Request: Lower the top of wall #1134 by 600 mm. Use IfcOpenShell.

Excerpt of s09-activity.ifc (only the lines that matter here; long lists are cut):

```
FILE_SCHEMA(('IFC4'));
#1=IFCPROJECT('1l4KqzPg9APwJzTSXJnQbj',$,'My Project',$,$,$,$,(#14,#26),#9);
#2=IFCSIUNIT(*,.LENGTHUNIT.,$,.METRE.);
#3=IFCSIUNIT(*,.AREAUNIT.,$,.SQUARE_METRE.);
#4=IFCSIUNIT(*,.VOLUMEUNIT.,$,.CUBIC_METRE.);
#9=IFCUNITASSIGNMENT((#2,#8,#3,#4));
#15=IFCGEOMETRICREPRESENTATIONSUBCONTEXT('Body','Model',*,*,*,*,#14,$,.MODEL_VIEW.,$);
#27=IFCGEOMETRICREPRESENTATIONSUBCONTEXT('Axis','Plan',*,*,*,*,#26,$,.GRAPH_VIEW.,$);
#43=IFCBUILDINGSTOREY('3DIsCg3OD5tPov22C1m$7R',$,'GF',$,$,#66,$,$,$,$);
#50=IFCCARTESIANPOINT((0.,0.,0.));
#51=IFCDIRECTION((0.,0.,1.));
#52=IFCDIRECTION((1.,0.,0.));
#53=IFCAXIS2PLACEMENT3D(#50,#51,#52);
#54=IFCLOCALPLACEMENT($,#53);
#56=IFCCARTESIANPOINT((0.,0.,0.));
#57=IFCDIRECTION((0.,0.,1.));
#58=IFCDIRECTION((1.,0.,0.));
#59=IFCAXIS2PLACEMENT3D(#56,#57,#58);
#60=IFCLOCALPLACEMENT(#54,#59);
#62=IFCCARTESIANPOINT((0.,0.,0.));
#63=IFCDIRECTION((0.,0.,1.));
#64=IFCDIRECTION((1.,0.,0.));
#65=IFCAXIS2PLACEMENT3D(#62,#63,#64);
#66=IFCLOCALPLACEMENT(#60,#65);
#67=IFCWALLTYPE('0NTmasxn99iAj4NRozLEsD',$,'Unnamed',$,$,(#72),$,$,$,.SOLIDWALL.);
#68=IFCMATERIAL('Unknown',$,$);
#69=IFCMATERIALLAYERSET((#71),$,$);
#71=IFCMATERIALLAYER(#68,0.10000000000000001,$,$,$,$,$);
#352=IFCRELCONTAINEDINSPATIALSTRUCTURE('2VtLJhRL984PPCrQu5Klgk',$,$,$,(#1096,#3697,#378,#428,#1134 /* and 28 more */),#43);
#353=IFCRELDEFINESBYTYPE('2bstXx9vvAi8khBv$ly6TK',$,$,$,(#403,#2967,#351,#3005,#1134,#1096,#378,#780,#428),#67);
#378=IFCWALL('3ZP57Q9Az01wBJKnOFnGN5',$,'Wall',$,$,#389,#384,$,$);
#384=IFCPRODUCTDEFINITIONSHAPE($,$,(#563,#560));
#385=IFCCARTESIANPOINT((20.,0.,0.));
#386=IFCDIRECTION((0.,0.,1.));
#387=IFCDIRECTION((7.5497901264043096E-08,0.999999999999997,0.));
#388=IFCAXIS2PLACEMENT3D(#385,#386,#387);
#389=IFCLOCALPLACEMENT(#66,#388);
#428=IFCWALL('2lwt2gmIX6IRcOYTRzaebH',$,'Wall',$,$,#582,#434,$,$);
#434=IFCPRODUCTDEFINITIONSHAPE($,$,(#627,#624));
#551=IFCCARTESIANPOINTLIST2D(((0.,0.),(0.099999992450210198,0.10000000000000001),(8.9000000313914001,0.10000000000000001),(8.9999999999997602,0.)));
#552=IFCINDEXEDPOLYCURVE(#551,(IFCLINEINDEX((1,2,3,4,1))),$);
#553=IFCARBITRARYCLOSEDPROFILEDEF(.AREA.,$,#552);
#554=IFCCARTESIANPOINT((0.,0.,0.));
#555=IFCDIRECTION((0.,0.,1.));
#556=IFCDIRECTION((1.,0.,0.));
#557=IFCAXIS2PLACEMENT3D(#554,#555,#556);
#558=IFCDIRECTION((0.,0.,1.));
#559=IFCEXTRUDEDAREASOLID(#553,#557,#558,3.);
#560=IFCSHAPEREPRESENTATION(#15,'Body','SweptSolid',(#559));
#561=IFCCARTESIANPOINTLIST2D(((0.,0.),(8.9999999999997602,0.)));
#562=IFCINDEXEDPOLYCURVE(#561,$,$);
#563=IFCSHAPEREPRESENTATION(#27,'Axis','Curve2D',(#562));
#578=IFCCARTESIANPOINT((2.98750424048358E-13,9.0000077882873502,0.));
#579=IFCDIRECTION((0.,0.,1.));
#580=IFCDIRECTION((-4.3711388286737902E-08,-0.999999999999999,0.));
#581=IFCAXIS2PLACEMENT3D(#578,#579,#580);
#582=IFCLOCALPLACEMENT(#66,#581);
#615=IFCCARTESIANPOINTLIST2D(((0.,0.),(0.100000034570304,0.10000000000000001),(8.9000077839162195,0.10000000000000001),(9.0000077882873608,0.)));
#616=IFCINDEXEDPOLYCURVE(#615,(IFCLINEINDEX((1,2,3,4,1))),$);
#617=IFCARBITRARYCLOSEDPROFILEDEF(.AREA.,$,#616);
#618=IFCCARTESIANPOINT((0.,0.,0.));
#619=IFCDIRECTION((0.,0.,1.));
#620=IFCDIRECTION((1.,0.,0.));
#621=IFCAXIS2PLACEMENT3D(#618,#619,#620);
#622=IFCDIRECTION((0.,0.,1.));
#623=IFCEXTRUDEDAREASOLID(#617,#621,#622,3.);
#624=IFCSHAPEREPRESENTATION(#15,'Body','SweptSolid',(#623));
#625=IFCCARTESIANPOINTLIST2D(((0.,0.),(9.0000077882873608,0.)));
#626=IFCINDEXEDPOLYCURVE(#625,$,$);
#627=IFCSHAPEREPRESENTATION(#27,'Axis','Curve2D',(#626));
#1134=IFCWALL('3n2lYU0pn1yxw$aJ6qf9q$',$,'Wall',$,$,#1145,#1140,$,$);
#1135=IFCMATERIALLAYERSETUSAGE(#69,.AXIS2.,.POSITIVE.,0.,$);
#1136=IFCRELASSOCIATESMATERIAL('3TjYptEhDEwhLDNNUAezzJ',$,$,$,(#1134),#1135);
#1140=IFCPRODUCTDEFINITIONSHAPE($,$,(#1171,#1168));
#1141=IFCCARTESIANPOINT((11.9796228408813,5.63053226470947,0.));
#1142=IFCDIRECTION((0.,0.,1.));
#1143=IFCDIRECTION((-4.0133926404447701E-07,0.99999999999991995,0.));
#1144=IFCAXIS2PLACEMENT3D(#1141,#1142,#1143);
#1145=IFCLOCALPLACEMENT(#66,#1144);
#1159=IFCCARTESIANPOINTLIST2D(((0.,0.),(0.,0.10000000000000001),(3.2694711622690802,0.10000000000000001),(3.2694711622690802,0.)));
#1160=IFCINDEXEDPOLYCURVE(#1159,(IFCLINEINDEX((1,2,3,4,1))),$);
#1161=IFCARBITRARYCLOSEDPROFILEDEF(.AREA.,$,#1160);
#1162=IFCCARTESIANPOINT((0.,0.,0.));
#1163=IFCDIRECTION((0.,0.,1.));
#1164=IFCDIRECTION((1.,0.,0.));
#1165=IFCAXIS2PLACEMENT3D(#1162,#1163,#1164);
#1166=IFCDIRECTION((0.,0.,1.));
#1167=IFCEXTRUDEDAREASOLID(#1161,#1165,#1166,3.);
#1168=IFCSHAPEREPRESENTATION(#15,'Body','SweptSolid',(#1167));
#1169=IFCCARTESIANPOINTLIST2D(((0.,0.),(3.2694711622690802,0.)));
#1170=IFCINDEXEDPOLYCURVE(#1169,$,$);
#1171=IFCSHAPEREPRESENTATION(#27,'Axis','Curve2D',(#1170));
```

```python
import ifcopenshell
import ifcopenshell.geom
import ifcopenshell.util.representation
import ifcopenshell.util.shape

model = ifcopenshell.open("s09-activity.ifc")
settings = ifcopenshell.geom.settings()


def volume(element):
    """Net volume in cubic metres, openings subtracted."""
    shape = ifcopenshell.geom.create_shape(settings, element)
    return ifcopenshell.util.shape.get_volume(shape.geometry)


wall = model.by_guid("3n2lYU0pn1yxw$aJ6qf9q$")
before = volume(wall)

body = ifcopenshell.util.representation.get_representation(wall, "Model", "Body")
solid = body.Items[0]
old_height = solid.Depth
solid.Depth -= 0.6
after = volume(wall)

print(f"height {old_height:g} -> {solid.Depth:g}, volume {before:.3f} -> {after:.3f} m3")

model.write("s09-activity_rev.ifc")
```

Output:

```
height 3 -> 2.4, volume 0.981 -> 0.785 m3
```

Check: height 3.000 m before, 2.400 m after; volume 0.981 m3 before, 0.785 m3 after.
